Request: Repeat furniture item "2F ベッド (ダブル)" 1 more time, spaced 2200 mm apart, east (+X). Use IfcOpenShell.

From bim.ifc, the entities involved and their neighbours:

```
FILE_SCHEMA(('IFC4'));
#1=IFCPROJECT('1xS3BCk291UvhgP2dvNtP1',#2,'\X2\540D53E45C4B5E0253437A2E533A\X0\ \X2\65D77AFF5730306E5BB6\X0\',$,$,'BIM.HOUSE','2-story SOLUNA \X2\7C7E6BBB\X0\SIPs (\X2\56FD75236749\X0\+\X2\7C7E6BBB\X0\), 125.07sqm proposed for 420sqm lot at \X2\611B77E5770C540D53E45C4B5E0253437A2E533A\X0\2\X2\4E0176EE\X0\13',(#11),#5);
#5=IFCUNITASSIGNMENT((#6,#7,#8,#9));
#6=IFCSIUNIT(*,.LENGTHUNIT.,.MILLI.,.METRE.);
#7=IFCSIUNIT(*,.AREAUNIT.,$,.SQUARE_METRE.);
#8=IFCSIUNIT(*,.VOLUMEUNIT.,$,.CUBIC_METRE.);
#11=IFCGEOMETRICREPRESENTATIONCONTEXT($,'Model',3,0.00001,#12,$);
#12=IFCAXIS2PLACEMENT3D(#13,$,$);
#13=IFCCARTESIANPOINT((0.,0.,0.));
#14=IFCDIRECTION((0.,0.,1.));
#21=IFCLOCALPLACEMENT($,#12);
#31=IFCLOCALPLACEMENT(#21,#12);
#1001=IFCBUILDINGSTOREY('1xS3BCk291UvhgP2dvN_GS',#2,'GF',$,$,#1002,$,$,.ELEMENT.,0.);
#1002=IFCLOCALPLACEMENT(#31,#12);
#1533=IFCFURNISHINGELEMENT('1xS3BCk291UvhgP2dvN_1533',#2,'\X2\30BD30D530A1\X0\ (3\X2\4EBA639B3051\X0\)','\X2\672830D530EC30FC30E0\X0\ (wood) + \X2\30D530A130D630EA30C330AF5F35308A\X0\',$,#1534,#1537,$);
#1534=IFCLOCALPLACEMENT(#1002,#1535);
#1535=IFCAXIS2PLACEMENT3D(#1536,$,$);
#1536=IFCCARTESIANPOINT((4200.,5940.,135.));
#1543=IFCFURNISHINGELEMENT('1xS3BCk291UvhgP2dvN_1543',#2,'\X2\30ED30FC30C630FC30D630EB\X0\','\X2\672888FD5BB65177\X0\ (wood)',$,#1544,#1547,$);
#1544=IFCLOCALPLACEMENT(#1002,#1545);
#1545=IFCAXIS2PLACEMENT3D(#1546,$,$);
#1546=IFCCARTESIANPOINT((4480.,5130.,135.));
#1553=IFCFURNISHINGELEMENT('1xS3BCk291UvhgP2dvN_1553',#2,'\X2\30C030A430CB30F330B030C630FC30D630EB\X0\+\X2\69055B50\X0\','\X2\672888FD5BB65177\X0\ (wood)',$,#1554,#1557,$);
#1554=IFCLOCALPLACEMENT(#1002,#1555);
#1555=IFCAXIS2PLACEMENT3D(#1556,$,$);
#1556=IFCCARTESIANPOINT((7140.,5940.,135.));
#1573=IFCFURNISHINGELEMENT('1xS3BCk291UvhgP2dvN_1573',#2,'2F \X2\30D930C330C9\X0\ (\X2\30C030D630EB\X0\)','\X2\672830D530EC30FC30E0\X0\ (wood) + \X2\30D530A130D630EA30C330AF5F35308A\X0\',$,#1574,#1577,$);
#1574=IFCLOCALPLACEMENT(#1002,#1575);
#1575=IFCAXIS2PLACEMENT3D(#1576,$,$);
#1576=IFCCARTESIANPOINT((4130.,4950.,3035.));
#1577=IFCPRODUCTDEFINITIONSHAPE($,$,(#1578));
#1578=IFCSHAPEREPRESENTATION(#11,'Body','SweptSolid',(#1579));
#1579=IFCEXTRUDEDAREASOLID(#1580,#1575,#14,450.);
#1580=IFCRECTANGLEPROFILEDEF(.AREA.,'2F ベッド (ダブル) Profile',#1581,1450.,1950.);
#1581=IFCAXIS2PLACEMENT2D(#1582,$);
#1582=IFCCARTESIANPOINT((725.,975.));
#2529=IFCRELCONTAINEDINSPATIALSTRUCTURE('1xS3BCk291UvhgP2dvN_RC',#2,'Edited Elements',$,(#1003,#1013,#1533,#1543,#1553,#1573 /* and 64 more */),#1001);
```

```python
import numpy as np
import ifcopenshell
import ifcopenshell.api.geometry
import ifcopenshell.api.root
import ifcopenshell.util.element
import ifcopenshell.util.placement
import ifcopenshell.util.unit

model = ifcopenshell.open("bim.ifc")
unit_scale = ifcopenshell.util.unit.calculate_unit_scale(model)


def reuse_history(source, copy):
    """copy_class also copies each property set's owner history, people and application; keep the originals."""
    for rel in copy.IsDefinedBy:
        if rel.is_a("IfcRelDefinesByProperties") and (history := rel.RelatingPropertyDefinition.OwnerHistory):
            rel.RelatingPropertyDefinition.OwnerHistory = source.OwnerHistory
            ifcopenshell.util.element.remove_deep2(model, history)


source = model.by_id(1573)
base = ifcopenshell.util.placement.get_local_placement(source.ObjectPlacement)
step = np.array([1.0, 0.0, 0.0]) * 2.2 / unit_scale

for i in range(1, 2):
    copy = ifcopenshell.api.root.copy_class(model, product=source)
    copy.Representation = ifcopenshell.util.element.copy_deep(
        model, source.Representation, exclude=["IfcGeometricRepresentationContext", "IfcRepresentationMap"]
    )
    reuse_history(source, copy)
    matrix = base.copy()
    matrix[:3, 3] += i * step
    print("added at", matrix[:3, 3].round(3) + 0.0)
    ifcopenshell.api.geometry.edit_object_placement(model, product=copy, matrix=matrix, is_si=False)

model.write("bim_updated.ifc")
```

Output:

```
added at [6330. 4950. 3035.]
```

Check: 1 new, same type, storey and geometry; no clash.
